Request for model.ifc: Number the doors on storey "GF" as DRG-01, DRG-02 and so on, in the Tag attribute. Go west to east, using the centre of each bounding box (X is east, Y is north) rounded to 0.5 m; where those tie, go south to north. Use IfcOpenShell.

First a look at what the model holds.

```python
import ifcopenshell
import ifcopenshell.util.element
import ifcopenshell.util.placement

model = ifcopenshell.open("model.ifc")
print(model.schema)
storey = next(s for s in model.by_type("IfcBuildingStorey") if s.Name == "GF")
doors = [e for e in ifcopenshell.util.element.get_decomposition(storey) if e.is_a("IfcDoor")]
for e in sorted(doors, key=lambda e: e.id()):
    origin = ifcopenshell.util.placement.get_local_placement(e.ObjectPlacement)[:3, 3]
    print(e.id(), e.Tag, e.Name, origin.round(2) + 0.0, sep=" | ")
```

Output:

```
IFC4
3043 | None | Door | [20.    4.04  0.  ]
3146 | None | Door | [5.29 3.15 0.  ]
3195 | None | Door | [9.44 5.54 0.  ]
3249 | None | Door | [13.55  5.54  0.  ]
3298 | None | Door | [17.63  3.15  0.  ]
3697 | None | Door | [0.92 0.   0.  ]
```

```python
import ifcopenshell
import ifcopenshell.geom
import ifcopenshell.util.element
import ifcopenshell.util.shape

model = ifcopenshell.open("model.ifc")
settings = ifcopenshell.geom.settings()
settings.set("use-world-coords", True)


def centre(element):
    shape = ifcopenshell.geom.create_shape(settings, element)
    return ifcopenshell.util.shape.get_bbox_centroid(shape.geometry)


storey = next(s for s in model.by_type("IfcBuildingStorey") if s.Name == "GF")
doors = [e for e in ifcopenshell.util.element.get_decomposition(storey) if e.is_a("IfcDoor")]

# Insertion points can sit at a corner or the storey origin, so sort by the geometry (in metres).
centres = {e: centre(e) for e in doors}
doors.sort(key=lambda e: (round(centres[e][0] / 0.5), centres[e][1]))

for i, e in enumerate(doors, start=1):
    number = f"DRG-{i:02d}"
    e.Tag = number
    print(e.id(), number)

model.write("model-out.ifc")
```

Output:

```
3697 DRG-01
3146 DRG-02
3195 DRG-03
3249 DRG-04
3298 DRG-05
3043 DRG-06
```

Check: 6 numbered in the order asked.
